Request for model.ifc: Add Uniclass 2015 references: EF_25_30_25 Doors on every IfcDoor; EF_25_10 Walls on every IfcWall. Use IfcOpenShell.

First a look at what the model holds.

```python
import ifcopenshell

model = ifcopenshell.open("model.ifc")
print(model.schema)
print("classifications:", [c.Name for c in model.by_type("IfcClassification")])
for ifc_class in ("IfcDoor", "IfcRoof", "IfcStair", "IfcWall", "IfcWindow"):
    print(ifc_class, len(model.by_type(ifc_class)))
```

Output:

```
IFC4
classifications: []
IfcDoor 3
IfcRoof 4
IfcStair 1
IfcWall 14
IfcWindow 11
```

```python
import ifcopenshell
import ifcopenshell.api.classification

model = ifcopenshell.open("model.ifc")

system = ifcopenshell.api.classification.add_classification(model, classification="Uniclass 2015")

codes = {
    "IfcDoor": ("EF_25_30_25", "Doors"),
    "IfcWall": ("EF_25_10", "Walls"),
}
for ifc_class, (code, name) in codes.items():
    products = model.by_type(ifc_class)
    ifcopenshell.api.classification.add_reference(
        model, products=products, classification=system, identification=code, name=name
    )
    print(code, len(products))

model.write("model-out.ifc")
```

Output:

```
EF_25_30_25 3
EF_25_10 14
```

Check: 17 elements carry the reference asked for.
